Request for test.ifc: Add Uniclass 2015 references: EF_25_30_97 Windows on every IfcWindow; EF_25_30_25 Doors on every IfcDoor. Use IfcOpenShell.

First a look at what the model holds.

```python
import ifcopenshell

model = ifcopenshell.open("test.ifc")
print(model.schema)
print("classifications:", [c.Name for c in model.by_type("IfcClassification")])
for ifc_class in ("IfcDoor", "IfcRoof", "IfcStair", "IfcWall", "IfcWindow"):
    print(ifc_class, len(model.by_type(ifc_class)))
```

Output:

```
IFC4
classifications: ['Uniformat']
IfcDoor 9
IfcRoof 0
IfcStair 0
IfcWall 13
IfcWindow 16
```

```python
import ifcopenshell
import ifcopenshell.api.classification

model = ifcopenshell.open("test.ifc")

system = ifcopenshell.api.classification.add_classification(model, classification="Uniclass 2015")

codes = {
    "IfcWindow": ("EF_25_30_97", "Windows"),
    "IfcDoor": ("EF_25_30_25", "Doors"),
}
for ifc_class, (code, name) in codes.items():
    products = model.by_type(ifc_class)
    ifcopenshell.api.classification.add_reference(
        model, products=products, classification=system, identification=code, name=name
    )
    print(code, len(products))

model.write("test_edited.ifc")
```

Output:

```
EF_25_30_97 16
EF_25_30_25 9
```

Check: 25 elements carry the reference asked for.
